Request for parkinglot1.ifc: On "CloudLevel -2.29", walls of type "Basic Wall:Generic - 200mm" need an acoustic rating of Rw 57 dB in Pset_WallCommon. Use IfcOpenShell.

First a look at what the model holds.

```python
import ifcopenshell
import ifcopenshell.util.element

model = ifcopenshell.open("parkinglot1.ifc")
print(model.schema)
storey = next(s for s in model.by_type("IfcBuildingStorey") if s.Name == "CloudLevel -2.29")
walls = [e for e in ifcopenshell.util.element.get_decomposition(storey) if e.is_a("IfcWall")]
seen = {}
for e in walls:
    element_type = ifcopenshell.util.element.get_type(e)
    key = (element_type.Name if element_type != e and element_type else None, ifcopenshell.util.element.get_pset(e, "Pset_WallCommon", "AcousticRating"))
    seen[key] = seen.get(key, 0) + 1
for (name, value), count in sorted(seen.items(), key=str):
    print(count, "x", name, "|", value)
```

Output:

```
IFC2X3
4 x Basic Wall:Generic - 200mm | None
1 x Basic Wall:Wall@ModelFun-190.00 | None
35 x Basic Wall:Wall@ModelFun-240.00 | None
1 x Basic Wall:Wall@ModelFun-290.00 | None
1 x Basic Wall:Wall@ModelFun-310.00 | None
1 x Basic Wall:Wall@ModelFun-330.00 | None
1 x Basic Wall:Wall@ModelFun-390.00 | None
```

```python
import ifcopenshell
import ifcopenshell.api.pset
import ifcopenshell.util.element

model = ifcopenshell.open("parkinglot1.ifc")

storey = next(s for s in model.by_type("IfcBuildingStorey") if s.Name == "CloudLevel -2.29")
walls = [e for e in ifcopenshell.util.element.get_decomposition(storey) if e.is_a("IfcWall")]

count = 0
for e in walls:
    element_type = ifcopenshell.util.element.get_type(e)
    if element_type in (None, e) or element_type.Name != "Basic Wall:Generic - 200mm":
        continue
    # add_pset returns the element's existing set when there is one.
    pset = ifcopenshell.api.pset.add_pset(model, product=e, name="Pset_WallCommon")
    ifcopenshell.api.pset.edit_pset(model, pset=pset, properties={"AcousticRating": "Rw 57 dB"})
    count += 1

print(count, "walls updated")

model.write("parkinglot1_rev.ifc")
```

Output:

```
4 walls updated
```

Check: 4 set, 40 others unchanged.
